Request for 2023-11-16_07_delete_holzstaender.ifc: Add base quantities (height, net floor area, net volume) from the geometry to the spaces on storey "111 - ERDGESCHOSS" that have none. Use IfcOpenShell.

First a look at what the model holds.

```python
import ifcopenshell
import ifcopenshell.util.element
import ifcopenshell.util.unit

model = ifcopenshell.open("2023-11-16_07_delete_holzstaender.ifc")
print(model.schema)
for unit_type in ("LENGTHUNIT", "AREAUNIT", "VOLUMEUNIT"):
    print(unit_type, ifcopenshell.util.unit.calculate_unit_scale(model, unit_type))
storey = next(s for s in model.by_type("IfcBuildingStorey") if s.Name == "111 - ERDGESCHOSS")
spaces = [e for e in ifcopenshell.util.element.get_decomposition(storey) if e.is_a("IfcSpace")]
for e in sorted(spaces, key=lambda e: e.id()):
    print(e.id(), e.is_a(), e.Name, list(ifcopenshell.util.element.get_psets(e, qtos_only=True)), sep=" | ")
```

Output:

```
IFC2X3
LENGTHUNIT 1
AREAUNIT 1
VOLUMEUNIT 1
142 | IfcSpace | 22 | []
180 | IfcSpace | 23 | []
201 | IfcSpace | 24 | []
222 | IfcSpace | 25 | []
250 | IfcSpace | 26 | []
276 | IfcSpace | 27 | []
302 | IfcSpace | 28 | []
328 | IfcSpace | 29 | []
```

```python
import ifcopenshell
import ifcopenshell.api.pset
import ifcopenshell.geom
import ifcopenshell.util.element
import ifcopenshell.util.shape
import ifcopenshell.util.unit

model = ifcopenshell.open("2023-11-16_07_delete_holzstaender.ifc")
unit_scale = ifcopenshell.util.unit.calculate_unit_scale(model)
area_scale = ifcopenshell.util.unit.calculate_unit_scale(model, "AREAUNIT")
volume_scale = ifcopenshell.util.unit.calculate_unit_scale(model, "VOLUMEUNIT")
settings = ifcopenshell.geom.settings()

storey = next(s for s in model.by_type("IfcBuildingStorey") if s.Name == "111 - ERDGESCHOSS")
spaces = [e for e in ifcopenshell.util.element.get_decomposition(storey) if e.is_a("IfcSpace")]

for e in sorted(spaces, key=lambda e: e.id()):
    if ifcopenshell.util.element.get_psets(e, qtos_only=True, should_inherit=False):
        continue
    # Geometry comes back in metres, in the element's own axes.
    shape = ifcopenshell.geom.create_shape(settings, e)
    values = {
        "Height": ifcopenshell.util.shape.get_z(shape.geometry) / unit_scale,
        "NetFloorArea": ifcopenshell.util.shape.get_footprint_area(shape.geometry) / area_scale,
        "NetVolume": ifcopenshell.util.shape.get_volume(shape.geometry) / volume_scale,
    }
    qto = ifcopenshell.api.pset.add_qto(model, product=e, name="BaseQuantities")
    ifcopenshell.api.pset.edit_qto(model, qto=qto, properties=values)
    print(e.id(), {k: round(v, 3) for k, v in values.items()})

model.write("2023-11-16_07_delete_holzstaender_v2.ifc")
```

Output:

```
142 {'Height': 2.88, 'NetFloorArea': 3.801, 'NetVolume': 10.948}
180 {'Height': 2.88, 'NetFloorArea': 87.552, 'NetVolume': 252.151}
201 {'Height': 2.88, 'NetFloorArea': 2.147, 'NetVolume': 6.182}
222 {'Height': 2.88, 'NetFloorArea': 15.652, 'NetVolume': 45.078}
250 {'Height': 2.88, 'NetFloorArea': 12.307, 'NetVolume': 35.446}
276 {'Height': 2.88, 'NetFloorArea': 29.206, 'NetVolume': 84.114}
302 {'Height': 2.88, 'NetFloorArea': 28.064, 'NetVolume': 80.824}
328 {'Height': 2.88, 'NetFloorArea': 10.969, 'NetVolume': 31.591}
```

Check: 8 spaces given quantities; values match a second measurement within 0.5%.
